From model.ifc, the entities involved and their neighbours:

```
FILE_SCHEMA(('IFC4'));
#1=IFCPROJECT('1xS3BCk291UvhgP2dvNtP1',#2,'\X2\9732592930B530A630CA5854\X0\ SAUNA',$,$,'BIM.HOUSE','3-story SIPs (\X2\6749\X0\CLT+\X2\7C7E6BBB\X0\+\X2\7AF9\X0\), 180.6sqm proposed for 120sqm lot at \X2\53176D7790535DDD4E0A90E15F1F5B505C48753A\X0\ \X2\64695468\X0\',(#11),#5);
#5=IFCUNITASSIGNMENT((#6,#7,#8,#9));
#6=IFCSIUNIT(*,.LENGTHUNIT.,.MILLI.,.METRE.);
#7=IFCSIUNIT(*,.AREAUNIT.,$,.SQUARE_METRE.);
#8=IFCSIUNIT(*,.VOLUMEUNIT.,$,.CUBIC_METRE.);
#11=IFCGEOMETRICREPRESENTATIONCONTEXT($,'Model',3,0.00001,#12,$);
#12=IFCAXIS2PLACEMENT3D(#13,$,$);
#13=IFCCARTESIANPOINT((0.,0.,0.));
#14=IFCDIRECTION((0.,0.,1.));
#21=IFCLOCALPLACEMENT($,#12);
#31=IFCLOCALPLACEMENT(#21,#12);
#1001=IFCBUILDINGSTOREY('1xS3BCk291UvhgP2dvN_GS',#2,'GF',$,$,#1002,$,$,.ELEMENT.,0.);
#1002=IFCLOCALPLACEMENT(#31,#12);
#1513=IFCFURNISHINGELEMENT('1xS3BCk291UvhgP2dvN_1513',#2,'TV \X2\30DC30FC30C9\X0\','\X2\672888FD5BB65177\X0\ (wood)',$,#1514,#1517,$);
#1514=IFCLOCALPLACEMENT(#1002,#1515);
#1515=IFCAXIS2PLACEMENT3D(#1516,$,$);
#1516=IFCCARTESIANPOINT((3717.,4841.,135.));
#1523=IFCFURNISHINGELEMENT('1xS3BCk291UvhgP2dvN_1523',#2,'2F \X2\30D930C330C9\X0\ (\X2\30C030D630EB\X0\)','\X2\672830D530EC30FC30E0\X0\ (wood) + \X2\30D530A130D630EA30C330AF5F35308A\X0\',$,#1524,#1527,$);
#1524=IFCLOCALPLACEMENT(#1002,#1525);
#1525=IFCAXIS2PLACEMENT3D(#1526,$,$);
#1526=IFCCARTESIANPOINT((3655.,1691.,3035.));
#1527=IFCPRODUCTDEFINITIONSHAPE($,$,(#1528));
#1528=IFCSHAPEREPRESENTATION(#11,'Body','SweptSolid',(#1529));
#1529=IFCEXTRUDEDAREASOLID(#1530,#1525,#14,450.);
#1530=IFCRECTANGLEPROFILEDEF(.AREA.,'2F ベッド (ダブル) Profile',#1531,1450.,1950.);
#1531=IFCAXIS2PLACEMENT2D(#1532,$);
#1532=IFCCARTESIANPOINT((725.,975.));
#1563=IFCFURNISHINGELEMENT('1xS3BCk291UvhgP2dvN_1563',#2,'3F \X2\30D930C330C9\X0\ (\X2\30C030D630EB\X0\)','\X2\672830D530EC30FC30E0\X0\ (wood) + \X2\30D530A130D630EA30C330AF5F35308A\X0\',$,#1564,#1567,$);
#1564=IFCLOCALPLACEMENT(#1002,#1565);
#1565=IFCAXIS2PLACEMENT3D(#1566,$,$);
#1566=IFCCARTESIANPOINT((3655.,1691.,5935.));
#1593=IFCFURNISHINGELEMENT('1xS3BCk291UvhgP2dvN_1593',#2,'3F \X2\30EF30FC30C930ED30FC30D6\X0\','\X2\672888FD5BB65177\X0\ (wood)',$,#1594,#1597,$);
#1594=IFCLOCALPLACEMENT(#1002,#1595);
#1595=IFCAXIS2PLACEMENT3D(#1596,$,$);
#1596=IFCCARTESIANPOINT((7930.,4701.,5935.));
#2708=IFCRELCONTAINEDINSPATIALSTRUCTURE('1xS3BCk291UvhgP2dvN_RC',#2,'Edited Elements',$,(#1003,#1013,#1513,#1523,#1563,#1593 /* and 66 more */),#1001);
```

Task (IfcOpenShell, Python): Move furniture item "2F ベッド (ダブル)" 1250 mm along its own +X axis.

```python
import ifcopenshell
import ifcopenshell.api.geometry
import ifcopenshell.util.placement

model = ifcopenshell.open("model.ifc")

item = model.by_guid("1xS3BCk291UvhgP2dvN_1523")
matrix = ifcopenshell.util.placement.get_local_placement(item.ObjectPlacement)
matrix[:3, 3] += matrix[:3, 0] * 1250.0
ifcopenshell.api.geometry.edit_object_placement(model, product=item, matrix=matrix, is_si=False)

print(ifcopenshell.util.placement.get_local_placement(item.ObjectPlacement).round(3) + 0.0)

model.write("model_updated.ifc")
```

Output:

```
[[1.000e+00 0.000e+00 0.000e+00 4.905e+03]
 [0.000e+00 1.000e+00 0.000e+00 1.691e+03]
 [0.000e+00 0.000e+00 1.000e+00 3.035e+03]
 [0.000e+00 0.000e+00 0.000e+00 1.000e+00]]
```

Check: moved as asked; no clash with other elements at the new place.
